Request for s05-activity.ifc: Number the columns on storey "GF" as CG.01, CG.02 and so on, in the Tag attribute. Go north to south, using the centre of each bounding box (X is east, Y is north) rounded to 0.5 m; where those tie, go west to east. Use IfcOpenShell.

First a look at what the model holds.

```python
import ifcopenshell
import ifcopenshell.util.element
import ifcopenshell.util.placement

model = ifcopenshell.open("s05-activity.ifc")
print(model.schema)
storey = next(s for s in model.by_type("IfcBuildingStorey") if s.Name == "GF")
columns = [e for e in ifcopenshell.util.element.get_decomposition(storey) if e.is_a("IfcColumn")]
for e in sorted(columns, key=lambda e: e.id()):
    origin = ifcopenshell.util.placement.get_local_placement(e.ObjectPlacement)[:3, 3]
    print(e.id(), e.Tag, e.Name, origin.round(2) + 0.0, sep=" | ")
```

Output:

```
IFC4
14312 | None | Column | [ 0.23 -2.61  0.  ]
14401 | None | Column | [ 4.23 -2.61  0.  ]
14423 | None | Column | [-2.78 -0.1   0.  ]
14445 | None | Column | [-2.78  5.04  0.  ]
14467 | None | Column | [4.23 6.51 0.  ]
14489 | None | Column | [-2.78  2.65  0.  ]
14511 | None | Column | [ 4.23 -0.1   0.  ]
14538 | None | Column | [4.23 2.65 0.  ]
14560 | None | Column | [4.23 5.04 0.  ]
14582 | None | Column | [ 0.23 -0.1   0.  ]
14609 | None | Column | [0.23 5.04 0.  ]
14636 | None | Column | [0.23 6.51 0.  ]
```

```python
import ifcopenshell
import ifcopenshell.geom
import ifcopenshell.util.element
import ifcopenshell.util.shape

model = ifcopenshell.open("s05-activity.ifc")
settings = ifcopenshell.geom.settings()
settings.set("use-world-coords", True)


def centre(element):
    shape = ifcopenshell.geom.create_shape(settings, element)
    return ifcopenshell.util.shape.get_bbox_centroid(shape.geometry)


storey = next(s for s in model.by_type("IfcBuildingStorey") if s.Name == "GF")
columns = [e for e in ifcopenshell.util.element.get_decomposition(storey) if e.is_a("IfcColumn")]

# Insertion points can sit at a corner or the storey origin, so sort by the geometry (in metres).
centres = {e: centre(e) for e in columns}
columns.sort(key=lambda e: (-round(centres[e][1] / 0.5), centres[e][0]))

for i, e in enumerate(columns, start=1):
    number = f"CG.{i:02d}"
    e.Tag = number
    print(e.id(), number)

model.write("s05-activity_v2.ifc")
```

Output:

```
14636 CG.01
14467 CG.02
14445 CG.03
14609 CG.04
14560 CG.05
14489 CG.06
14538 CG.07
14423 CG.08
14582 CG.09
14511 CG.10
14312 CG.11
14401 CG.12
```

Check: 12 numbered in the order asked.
